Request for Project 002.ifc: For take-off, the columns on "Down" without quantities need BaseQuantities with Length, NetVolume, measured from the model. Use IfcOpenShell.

First a look at what the model holds.

```python
import ifcopenshell
import ifcopenshell.util.element
import ifcopenshell.util.unit

model = ifcopenshell.open("Project 002.ifc")
print(model.schema)
for unit_type in ("LENGTHUNIT", "AREAUNIT", "VOLUMEUNIT"):
    print(unit_type, ifcopenshell.util.unit.calculate_unit_scale(model, unit_type))
storey = next(s for s in model.by_type("IfcBuildingStorey") if s.Name == "Down")
columns = [e for e in ifcopenshell.util.element.get_decomposition(storey) if e.is_a("IfcColumn")]
for e in sorted(columns, key=lambda e: e.id()):
    print(e.id(), e.is_a(), e.Name, list(ifcopenshell.util.element.get_psets(e, qtos_only=True)), sep=" | ")
```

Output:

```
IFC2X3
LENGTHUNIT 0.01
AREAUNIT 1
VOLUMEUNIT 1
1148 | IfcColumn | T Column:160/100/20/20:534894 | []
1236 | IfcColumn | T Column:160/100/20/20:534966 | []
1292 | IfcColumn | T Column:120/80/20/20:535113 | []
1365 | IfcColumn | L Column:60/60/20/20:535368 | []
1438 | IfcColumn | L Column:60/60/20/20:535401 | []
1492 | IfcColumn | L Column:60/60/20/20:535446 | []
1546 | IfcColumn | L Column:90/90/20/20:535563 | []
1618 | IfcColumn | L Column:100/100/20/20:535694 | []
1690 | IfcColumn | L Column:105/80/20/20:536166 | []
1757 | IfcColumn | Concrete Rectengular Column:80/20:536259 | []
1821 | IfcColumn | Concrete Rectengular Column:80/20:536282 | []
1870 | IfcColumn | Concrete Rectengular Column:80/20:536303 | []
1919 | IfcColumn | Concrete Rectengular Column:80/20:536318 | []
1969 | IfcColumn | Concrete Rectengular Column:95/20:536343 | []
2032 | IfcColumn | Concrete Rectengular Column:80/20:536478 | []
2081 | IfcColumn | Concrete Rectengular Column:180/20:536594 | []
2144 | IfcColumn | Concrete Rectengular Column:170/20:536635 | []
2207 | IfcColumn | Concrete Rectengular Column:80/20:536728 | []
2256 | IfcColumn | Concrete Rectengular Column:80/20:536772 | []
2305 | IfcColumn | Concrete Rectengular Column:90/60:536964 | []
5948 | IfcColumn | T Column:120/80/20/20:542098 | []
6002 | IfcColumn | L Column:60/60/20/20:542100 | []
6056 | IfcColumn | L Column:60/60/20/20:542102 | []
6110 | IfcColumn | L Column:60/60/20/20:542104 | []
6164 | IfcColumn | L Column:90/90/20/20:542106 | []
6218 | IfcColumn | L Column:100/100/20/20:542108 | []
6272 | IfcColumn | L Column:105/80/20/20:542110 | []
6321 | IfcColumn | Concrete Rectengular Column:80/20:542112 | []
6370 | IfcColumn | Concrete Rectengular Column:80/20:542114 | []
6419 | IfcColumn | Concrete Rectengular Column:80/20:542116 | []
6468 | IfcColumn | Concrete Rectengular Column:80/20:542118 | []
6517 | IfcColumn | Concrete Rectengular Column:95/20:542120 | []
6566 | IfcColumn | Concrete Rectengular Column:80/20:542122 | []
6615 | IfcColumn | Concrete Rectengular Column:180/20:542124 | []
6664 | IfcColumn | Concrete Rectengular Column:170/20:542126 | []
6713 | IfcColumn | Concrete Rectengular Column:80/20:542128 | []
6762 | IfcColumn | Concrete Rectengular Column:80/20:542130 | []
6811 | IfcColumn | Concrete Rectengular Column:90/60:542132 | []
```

```python
import ifcopenshell
import ifcopenshell.api.pset
import ifcopenshell.geom
import ifcopenshell.util.element
import ifcopenshell.util.shape
import ifcopenshell.util.unit

model = ifcopenshell.open("Project 002.ifc")
unit_scale = ifcopenshell.util.unit.calculate_unit_scale(model)
volume_scale = ifcopenshell.util.unit.calculate_unit_scale(model, "VOLUMEUNIT")
settings = ifcopenshell.geom.settings()

storey = next(s for s in model.by_type("IfcBuildingStorey") if s.Name == "Down")
columns = [e for e in ifcopenshell.util.element.get_decomposition(storey) if e.is_a("IfcColumn")]

for e in sorted(columns, key=lambda e: e.id()):
    if ifcopenshell.util.element.get_psets(e, qtos_only=True, should_inherit=False):
        continue
    # Geometry comes back in metres, in the element's own axes.
    shape = ifcopenshell.geom.create_shape(settings, e)
    values = {
        "Length": ifcopenshell.util.shape.get_z(shape.geometry) / unit_scale,
        "NetVolume": ifcopenshell.util.shape.get_volume(shape.geometry) / volume_scale,
    }
    qto = ifcopenshell.api.pset.add_qto(model, product=e, name="BaseQuantities")
    ifcopenshell.api.pset.edit_qto(model, qto=qto, properties=values)
    print(e.id(), {k: round(v, 3) for k, v in values.items()})

model.write("Project 002_v2.ifc")
```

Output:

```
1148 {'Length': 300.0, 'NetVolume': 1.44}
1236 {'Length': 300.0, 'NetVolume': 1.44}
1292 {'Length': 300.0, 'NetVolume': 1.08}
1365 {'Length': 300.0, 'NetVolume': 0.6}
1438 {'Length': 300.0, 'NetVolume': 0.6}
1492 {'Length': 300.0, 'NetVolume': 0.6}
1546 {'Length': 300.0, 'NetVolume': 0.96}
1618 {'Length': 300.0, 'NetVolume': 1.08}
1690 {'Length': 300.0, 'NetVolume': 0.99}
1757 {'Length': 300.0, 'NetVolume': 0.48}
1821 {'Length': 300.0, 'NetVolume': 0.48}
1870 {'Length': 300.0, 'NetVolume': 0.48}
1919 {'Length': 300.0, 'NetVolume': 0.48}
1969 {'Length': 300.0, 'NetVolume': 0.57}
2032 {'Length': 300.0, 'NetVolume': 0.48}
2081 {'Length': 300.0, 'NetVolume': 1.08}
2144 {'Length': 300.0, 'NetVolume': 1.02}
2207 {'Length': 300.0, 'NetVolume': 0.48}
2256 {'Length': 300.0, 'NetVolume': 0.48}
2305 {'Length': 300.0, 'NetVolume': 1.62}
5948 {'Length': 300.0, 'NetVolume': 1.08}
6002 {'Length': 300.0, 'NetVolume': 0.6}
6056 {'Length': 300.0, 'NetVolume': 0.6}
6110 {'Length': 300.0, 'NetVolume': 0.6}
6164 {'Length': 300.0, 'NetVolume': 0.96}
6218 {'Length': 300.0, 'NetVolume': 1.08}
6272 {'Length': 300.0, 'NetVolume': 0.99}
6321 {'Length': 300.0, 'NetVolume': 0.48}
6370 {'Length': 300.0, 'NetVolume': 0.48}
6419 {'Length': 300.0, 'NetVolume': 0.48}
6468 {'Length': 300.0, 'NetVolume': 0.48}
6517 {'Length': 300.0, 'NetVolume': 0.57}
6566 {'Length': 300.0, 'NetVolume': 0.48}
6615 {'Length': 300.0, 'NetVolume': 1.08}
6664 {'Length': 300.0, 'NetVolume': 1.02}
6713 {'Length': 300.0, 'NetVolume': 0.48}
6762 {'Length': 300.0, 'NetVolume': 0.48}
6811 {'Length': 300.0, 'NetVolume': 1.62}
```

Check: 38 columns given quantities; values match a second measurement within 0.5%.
